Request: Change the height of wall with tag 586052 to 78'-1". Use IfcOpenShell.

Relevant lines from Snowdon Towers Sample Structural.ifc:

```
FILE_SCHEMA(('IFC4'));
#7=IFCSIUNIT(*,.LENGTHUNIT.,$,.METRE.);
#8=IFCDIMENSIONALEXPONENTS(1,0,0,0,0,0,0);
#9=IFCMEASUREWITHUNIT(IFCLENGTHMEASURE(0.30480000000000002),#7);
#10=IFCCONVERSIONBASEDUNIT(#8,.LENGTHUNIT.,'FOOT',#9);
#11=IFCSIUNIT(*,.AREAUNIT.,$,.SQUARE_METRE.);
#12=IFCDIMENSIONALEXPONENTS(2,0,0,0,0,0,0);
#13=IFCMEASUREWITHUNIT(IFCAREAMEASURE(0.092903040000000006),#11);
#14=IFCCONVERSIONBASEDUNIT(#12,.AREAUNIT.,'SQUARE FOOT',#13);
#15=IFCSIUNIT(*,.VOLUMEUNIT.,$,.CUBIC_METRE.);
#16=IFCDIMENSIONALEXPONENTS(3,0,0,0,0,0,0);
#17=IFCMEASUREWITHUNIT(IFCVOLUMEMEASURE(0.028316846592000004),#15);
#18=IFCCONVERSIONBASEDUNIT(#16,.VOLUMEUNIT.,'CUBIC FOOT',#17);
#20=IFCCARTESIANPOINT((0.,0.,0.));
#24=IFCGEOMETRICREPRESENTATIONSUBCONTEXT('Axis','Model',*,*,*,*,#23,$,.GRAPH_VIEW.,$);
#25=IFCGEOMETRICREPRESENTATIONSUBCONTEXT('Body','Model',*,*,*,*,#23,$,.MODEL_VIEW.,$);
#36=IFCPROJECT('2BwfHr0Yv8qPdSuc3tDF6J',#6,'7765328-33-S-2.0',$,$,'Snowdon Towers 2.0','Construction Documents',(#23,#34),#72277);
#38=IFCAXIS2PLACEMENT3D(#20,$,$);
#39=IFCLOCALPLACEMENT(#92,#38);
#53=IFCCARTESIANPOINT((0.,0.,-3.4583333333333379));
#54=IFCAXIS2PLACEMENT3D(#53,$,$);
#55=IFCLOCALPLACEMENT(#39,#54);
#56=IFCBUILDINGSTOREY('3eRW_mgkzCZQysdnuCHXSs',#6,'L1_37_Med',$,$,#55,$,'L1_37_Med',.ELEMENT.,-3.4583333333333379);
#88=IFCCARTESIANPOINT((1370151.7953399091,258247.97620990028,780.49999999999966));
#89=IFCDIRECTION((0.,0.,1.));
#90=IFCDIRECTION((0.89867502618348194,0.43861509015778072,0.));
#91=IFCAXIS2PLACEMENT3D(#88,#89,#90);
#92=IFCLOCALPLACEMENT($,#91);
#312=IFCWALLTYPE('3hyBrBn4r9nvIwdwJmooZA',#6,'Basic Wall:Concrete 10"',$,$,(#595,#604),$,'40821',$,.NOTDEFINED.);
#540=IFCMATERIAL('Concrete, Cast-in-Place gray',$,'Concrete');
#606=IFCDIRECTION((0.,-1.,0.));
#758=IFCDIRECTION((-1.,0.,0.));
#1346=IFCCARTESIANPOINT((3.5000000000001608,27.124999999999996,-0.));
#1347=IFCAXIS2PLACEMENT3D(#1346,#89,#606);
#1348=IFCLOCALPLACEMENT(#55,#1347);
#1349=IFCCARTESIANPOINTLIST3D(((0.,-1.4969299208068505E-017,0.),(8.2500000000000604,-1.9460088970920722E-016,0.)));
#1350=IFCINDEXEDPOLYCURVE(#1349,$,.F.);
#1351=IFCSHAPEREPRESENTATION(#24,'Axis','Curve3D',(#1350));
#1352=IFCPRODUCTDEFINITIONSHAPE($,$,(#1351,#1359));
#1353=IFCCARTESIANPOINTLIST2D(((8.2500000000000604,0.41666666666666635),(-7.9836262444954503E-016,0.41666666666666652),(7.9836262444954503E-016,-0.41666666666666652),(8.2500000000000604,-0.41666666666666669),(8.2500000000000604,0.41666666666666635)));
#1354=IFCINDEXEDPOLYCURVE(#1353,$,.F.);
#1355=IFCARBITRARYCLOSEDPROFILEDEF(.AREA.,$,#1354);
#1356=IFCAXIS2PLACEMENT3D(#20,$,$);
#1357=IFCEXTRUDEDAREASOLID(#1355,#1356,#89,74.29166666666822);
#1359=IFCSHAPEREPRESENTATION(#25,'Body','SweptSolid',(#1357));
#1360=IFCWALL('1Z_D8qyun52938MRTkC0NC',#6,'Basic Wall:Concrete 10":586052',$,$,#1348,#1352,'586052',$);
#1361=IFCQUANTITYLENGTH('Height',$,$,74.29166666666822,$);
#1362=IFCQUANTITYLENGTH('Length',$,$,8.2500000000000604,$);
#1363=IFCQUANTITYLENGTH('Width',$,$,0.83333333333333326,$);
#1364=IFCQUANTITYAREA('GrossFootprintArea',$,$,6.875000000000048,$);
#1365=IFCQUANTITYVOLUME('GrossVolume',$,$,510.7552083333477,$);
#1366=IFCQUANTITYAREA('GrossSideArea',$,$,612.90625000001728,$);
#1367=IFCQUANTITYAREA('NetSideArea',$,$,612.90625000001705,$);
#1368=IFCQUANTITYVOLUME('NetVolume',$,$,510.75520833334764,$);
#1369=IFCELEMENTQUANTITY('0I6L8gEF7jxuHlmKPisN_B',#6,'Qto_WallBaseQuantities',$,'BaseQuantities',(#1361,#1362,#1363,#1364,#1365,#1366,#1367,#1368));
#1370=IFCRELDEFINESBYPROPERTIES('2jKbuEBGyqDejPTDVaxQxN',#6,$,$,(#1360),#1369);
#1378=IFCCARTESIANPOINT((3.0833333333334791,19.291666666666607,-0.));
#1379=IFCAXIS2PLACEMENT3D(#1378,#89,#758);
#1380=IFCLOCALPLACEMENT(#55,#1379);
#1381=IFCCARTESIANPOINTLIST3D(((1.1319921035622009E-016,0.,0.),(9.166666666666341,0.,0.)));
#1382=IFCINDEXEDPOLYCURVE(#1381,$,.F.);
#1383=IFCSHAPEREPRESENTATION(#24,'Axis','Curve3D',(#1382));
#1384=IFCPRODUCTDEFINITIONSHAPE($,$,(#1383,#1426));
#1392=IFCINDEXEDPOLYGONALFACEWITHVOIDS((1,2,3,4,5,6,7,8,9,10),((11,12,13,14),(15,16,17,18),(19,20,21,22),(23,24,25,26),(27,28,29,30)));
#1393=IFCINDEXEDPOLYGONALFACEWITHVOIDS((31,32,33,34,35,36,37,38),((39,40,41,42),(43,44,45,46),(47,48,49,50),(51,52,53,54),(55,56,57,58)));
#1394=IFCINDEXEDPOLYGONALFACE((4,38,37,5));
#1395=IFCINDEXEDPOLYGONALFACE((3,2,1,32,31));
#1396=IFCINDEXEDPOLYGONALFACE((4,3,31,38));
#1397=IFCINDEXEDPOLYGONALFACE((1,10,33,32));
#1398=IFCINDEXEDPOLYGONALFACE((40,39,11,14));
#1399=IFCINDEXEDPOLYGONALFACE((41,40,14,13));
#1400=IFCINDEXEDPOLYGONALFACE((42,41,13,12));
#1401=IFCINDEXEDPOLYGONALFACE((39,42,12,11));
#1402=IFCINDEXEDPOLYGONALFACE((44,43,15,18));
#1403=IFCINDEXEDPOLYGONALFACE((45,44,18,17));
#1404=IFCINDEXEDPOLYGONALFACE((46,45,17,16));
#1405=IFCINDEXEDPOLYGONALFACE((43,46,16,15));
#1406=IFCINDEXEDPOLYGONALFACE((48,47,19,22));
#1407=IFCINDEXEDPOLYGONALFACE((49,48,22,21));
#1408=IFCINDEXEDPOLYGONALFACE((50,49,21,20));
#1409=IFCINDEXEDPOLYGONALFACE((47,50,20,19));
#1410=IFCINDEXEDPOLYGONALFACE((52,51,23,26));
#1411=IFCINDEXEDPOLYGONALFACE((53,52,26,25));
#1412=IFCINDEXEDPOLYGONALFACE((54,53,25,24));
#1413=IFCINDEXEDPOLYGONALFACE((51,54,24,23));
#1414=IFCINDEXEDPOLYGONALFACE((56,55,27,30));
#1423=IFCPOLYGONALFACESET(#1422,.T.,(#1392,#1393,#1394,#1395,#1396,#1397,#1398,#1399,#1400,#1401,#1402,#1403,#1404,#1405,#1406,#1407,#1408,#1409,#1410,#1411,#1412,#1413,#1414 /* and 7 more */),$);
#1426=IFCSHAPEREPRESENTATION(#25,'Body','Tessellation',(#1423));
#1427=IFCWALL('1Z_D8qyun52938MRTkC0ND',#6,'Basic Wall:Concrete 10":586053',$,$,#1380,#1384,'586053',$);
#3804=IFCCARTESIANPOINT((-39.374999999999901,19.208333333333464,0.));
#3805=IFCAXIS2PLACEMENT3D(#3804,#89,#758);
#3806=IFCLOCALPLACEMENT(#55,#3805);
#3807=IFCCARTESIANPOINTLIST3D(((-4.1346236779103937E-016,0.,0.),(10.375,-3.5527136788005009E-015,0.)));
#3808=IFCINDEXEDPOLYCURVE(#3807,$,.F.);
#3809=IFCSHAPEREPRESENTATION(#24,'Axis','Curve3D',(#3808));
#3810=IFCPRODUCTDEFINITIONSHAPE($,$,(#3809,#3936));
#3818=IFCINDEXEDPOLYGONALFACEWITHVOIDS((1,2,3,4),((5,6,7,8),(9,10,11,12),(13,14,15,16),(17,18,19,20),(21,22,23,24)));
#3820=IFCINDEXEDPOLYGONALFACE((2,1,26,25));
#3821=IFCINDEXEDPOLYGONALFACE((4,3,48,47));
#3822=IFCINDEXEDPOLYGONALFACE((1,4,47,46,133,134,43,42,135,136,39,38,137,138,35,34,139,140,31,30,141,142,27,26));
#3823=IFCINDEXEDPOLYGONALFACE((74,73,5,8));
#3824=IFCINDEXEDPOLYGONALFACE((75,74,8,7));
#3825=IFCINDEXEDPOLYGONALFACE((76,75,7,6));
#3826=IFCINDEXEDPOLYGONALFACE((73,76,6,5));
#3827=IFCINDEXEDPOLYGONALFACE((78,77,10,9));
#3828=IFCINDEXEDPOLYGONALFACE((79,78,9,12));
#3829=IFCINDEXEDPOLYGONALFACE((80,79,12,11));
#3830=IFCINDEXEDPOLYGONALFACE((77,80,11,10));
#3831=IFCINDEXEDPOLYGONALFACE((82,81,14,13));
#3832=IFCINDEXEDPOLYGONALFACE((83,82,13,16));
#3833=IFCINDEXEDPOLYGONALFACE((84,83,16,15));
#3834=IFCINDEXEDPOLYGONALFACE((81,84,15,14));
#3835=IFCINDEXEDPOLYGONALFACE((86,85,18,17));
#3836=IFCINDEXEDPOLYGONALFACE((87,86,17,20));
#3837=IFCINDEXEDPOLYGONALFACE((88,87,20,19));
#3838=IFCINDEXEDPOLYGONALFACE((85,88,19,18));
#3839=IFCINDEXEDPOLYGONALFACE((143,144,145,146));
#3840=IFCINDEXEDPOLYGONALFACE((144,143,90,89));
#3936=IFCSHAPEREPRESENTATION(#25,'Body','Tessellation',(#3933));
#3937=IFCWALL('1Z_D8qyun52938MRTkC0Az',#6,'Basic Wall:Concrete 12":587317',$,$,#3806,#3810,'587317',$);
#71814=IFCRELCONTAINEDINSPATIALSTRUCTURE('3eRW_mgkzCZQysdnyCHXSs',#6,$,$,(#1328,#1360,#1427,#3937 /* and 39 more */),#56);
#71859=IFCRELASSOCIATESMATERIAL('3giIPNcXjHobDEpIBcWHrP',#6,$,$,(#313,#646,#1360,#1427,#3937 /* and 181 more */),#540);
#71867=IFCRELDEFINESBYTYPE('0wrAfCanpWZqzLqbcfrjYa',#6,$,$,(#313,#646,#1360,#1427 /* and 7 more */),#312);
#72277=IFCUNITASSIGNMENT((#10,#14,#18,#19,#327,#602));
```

```python
import ifcopenshell
import ifcopenshell.api.pset
import ifcopenshell.geom
import ifcopenshell.util.element
import ifcopenshell.util.representation
import ifcopenshell.util.shape
import ifcopenshell.util.unit

model = ifcopenshell.open("Snowdon Towers Sample Structural.ifc")
unit_scale = ifcopenshell.util.unit.calculate_unit_scale(model)
area_scale = ifcopenshell.util.unit.calculate_unit_scale(model, "AREAUNIT")
volume_scale = ifcopenshell.util.unit.calculate_unit_scale(model, "VOLUMEUNIT")
settings = ifcopenshell.geom.settings()


def volume(element):
    """Net volume in cubic metres, openings subtracted."""
    shape = ifcopenshell.geom.create_shape(settings, element)
    return ifcopenshell.util.shape.get_volume(shape.geometry)


wall = model.by_guid("1Z_D8qyun52938MRTkC0NC")
before = volume(wall)

body = ifcopenshell.util.representation.get_representation(wall, "Model", "Body")
solid = body.Items[0]
old_height = solid.Depth
solid.Depth = 937 * 0.0254 / unit_scale
after = volume(wall)
thickness = 0.254  # wall thickness in metres

# Update the stored height, areas and volumes.
qto = model.by_id(ifcopenshell.util.element.get_pset(wall, "Qto_WallBaseQuantities", should_inherit=False)["id"])
ifcopenshell.api.pset.edit_qto(model, qto=qto, properties={
    "Height": solid.Depth,
    "GrossVolume": ifcopenshell.util.element.get_pset(wall, "Qto_WallBaseQuantities", "GrossVolume") * solid.Depth / old_height,
    "GrossSideArea": ifcopenshell.util.element.get_pset(wall, "Qto_WallBaseQuantities", "GrossSideArea") * solid.Depth / old_height,
    "NetSideArea": after / thickness / area_scale,
    "NetVolume": after / volume_scale,
})

print(f"height {old_height:g} -> {solid.Depth:g}, volume {before:.3f} -> {after:.3f} m3")

model.write("Snowdon Towers Sample Structural_updated.ifc")
```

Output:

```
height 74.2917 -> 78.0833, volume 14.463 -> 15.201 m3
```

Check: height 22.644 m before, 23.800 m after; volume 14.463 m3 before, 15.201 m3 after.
